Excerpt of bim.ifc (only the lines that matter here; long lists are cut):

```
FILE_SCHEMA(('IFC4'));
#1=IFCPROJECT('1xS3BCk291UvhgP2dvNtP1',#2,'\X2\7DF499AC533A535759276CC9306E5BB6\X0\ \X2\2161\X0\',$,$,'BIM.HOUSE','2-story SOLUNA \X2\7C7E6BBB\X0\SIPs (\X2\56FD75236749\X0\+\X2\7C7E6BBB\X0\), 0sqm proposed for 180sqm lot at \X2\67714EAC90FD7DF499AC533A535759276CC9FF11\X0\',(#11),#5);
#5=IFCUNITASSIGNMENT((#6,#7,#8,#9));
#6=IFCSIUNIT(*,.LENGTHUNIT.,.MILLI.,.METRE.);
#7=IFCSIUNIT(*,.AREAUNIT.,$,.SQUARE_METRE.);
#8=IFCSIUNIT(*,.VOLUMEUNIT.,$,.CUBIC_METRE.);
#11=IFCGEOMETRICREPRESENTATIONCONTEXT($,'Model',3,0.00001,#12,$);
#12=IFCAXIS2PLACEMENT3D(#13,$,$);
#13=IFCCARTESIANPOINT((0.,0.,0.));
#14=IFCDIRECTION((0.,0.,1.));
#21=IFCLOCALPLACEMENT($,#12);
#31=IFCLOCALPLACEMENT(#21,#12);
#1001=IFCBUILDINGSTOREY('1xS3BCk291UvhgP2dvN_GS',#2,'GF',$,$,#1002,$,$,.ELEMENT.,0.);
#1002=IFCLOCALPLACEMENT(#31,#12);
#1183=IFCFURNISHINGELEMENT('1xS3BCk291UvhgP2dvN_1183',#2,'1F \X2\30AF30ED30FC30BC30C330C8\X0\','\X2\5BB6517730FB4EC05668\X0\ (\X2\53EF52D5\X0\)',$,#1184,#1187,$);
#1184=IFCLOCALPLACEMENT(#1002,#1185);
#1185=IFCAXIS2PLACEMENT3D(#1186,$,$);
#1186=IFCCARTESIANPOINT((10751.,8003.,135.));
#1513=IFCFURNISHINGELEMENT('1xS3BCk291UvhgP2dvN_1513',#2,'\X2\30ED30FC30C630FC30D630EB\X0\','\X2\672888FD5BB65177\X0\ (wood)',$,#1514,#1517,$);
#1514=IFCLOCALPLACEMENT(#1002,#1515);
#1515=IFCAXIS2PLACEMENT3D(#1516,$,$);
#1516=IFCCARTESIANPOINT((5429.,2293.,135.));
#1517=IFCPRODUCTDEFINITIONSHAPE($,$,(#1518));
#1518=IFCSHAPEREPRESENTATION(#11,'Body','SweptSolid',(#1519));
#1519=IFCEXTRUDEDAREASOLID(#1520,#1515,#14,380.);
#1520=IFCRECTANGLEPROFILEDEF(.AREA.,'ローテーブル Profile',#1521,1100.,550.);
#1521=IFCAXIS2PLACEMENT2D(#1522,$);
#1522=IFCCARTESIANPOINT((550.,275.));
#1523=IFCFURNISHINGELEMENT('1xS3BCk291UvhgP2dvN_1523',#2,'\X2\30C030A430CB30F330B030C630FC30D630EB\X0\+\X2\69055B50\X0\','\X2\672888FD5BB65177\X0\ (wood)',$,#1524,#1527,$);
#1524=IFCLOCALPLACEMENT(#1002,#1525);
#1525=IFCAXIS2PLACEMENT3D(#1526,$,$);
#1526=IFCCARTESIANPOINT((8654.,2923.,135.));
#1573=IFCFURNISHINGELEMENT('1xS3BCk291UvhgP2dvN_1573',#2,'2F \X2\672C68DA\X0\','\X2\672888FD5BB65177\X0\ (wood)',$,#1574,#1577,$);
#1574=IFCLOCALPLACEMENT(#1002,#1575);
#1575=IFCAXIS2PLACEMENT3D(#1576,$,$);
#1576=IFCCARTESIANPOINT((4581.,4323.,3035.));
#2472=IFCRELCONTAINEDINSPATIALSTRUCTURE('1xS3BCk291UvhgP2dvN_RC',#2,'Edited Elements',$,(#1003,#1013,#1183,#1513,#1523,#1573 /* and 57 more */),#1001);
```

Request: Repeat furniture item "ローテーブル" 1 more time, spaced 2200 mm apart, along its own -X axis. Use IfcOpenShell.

```python
import ifcopenshell
import ifcopenshell.api.geometry
import ifcopenshell.api.root
import ifcopenshell.util.element
import ifcopenshell.util.placement

model = ifcopenshell.open("bim.ifc")


def reuse_history(source, copy):
    """copy_class also copies each property set's owner history, people and application; keep the originals."""
    for rel in copy.IsDefinedBy:
        if rel.is_a("IfcRelDefinesByProperties") and (history := rel.RelatingPropertyDefinition.OwnerHistory):
            rel.RelatingPropertyDefinition.OwnerHistory = source.OwnerHistory
            ifcopenshell.util.element.remove_deep2(model, history)


source = model.by_guid("1xS3BCk291UvhgP2dvN_1513")
base = ifcopenshell.util.placement.get_local_placement(source.ObjectPlacement)
step = -base[:3, 0] * 2200.0

for i in range(1, 2):
    copy = ifcopenshell.api.root.copy_class(model, product=source)
    copy.Representation = ifcopenshell.util.element.copy_deep(
        model, source.Representation, exclude=["IfcGeometricRepresentationContext", "IfcRepresentationMap"]
    )
    reuse_history(source, copy)
    matrix = base.copy()
    matrix[:3, 3] += i * step
    print("added at", matrix[:3, 3].round(3) + 0.0)
    ifcopenshell.api.geometry.edit_object_placement(model, product=copy, matrix=matrix, is_si=False)

model.write("bim_v2.ifc")
```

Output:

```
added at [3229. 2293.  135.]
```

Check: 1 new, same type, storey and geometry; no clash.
